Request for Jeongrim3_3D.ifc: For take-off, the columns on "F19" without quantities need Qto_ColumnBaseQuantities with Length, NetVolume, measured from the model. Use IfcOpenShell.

First a look at what the model holds.

```python
import ifcopenshell
import ifcopenshell.util.element
import ifcopenshell.util.unit

model = ifcopenshell.open("Jeongrim3_3D.ifc")
print(model.schema)
for unit_type in ("LENGTHUNIT", "AREAUNIT", "VOLUMEUNIT"):
    print(unit_type, ifcopenshell.util.unit.calculate_unit_scale(model, unit_type))
storey = next(s for s in model.by_type("IfcBuildingStorey") if s.Name == "F19")
columns = [e for e in ifcopenshell.util.element.get_decomposition(storey) if e.is_a("IfcColumn")]
for e in sorted(columns, key=lambda e: e.id()):
    print(e.id(), e.is_a(), e.Name, list(ifcopenshell.util.element.get_psets(e, qtos_only=True)), sep=" | ")
```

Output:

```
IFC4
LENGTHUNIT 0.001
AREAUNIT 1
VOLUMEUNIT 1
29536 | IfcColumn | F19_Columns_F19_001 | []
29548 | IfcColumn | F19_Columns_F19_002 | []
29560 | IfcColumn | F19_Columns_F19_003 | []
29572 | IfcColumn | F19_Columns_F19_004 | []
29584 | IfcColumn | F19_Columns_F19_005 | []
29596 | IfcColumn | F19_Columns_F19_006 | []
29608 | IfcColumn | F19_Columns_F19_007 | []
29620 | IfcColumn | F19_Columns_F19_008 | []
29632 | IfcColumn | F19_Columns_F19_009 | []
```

```python
import ifcopenshell
import ifcopenshell.api.pset
import ifcopenshell.geom
import ifcopenshell.util.element
import ifcopenshell.util.shape
import ifcopenshell.util.unit

model = ifcopenshell.open("Jeongrim3_3D.ifc")
unit_scale = ifcopenshell.util.unit.calculate_unit_scale(model)
volume_scale = ifcopenshell.util.unit.calculate_unit_scale(model, "VOLUMEUNIT")
settings = ifcopenshell.geom.settings()

storey = next(s for s in model.by_type("IfcBuildingStorey") if s.Name == "F19")
columns = [e for e in ifcopenshell.util.element.get_decomposition(storey) if e.is_a("IfcColumn")]

for e in sorted(columns, key=lambda e: e.id()):
    if ifcopenshell.util.element.get_psets(e, qtos_only=True, should_inherit=False):
        continue
    # Geometry comes back in metres, in the element's own axes.
    shape = ifcopenshell.geom.create_shape(settings, e)
    values = {
        "Length": ifcopenshell.util.shape.get_z(shape.geometry) / unit_scale,
        "NetVolume": ifcopenshell.util.shape.get_volume(shape.geometry) / volume_scale,
    }
    qto = ifcopenshell.api.pset.add_qto(model, product=e, name="Qto_ColumnBaseQuantities")
    ifcopenshell.api.pset.edit_qto(model, qto=qto, properties=values)
    print(e.id(), {k: round(v, 3) for k, v in values.items()})

model.write("Jeongrim3_3D_edited.ifc")
```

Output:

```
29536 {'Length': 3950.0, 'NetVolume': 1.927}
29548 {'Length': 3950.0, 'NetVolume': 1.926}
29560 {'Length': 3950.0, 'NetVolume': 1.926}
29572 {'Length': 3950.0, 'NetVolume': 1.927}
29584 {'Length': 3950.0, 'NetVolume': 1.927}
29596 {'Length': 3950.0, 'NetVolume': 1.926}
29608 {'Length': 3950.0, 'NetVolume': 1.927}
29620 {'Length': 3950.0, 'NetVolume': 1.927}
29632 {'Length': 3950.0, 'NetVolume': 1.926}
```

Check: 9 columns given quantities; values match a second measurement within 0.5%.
